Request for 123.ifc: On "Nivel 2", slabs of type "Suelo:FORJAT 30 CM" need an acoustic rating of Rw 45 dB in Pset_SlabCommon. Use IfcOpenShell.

First a look at what the model holds.

```python
import ifcopenshell
import ifcopenshell.util.element

model = ifcopenshell.open("123.ifc")
print(model.schema)
storey = next(s for s in model.by_type("IfcBuildingStorey") if s.Name == "Nivel 2")
slabs = [e for e in ifcopenshell.util.element.get_decomposition(storey) if e.is_a("IfcSlab")]
seen = {}
for e in slabs:
    element_type = ifcopenshell.util.element.get_type(e)
    key = (element_type.Name if element_type != e and element_type else None, ifcopenshell.util.element.get_pset(e, "Pset_SlabCommon", "AcousticRating"))
    seen[key] = seen.get(key, 0) + 1
for (name, value), count in sorted(seen.items(), key=str):
    print(count, "x", name, "|", value)
```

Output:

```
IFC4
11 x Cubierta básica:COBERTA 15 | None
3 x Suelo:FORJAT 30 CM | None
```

```python
import ifcopenshell
import ifcopenshell.api.pset
import ifcopenshell.util.element

model = ifcopenshell.open("123.ifc")

storey = next(s for s in model.by_type("IfcBuildingStorey") if s.Name == "Nivel 2")
slabs = [e for e in ifcopenshell.util.element.get_decomposition(storey) if e.is_a("IfcSlab")]

count = 0
for e in slabs:
    element_type = ifcopenshell.util.element.get_type(e)
    if element_type in (None, e) or element_type.Name != "Suelo:FORJAT 30 CM":
        continue
    # add_pset returns the element's existing set when there is one.
    pset = ifcopenshell.api.pset.add_pset(model, product=e, name="Pset_SlabCommon")
    ifcopenshell.api.pset.edit_pset(model, pset=pset, properties={"AcousticRating": "Rw 45 dB"})
    count += 1

print(count, "slabs updated")

model.write("123_rev.ifc")
```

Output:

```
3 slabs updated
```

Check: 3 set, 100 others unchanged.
